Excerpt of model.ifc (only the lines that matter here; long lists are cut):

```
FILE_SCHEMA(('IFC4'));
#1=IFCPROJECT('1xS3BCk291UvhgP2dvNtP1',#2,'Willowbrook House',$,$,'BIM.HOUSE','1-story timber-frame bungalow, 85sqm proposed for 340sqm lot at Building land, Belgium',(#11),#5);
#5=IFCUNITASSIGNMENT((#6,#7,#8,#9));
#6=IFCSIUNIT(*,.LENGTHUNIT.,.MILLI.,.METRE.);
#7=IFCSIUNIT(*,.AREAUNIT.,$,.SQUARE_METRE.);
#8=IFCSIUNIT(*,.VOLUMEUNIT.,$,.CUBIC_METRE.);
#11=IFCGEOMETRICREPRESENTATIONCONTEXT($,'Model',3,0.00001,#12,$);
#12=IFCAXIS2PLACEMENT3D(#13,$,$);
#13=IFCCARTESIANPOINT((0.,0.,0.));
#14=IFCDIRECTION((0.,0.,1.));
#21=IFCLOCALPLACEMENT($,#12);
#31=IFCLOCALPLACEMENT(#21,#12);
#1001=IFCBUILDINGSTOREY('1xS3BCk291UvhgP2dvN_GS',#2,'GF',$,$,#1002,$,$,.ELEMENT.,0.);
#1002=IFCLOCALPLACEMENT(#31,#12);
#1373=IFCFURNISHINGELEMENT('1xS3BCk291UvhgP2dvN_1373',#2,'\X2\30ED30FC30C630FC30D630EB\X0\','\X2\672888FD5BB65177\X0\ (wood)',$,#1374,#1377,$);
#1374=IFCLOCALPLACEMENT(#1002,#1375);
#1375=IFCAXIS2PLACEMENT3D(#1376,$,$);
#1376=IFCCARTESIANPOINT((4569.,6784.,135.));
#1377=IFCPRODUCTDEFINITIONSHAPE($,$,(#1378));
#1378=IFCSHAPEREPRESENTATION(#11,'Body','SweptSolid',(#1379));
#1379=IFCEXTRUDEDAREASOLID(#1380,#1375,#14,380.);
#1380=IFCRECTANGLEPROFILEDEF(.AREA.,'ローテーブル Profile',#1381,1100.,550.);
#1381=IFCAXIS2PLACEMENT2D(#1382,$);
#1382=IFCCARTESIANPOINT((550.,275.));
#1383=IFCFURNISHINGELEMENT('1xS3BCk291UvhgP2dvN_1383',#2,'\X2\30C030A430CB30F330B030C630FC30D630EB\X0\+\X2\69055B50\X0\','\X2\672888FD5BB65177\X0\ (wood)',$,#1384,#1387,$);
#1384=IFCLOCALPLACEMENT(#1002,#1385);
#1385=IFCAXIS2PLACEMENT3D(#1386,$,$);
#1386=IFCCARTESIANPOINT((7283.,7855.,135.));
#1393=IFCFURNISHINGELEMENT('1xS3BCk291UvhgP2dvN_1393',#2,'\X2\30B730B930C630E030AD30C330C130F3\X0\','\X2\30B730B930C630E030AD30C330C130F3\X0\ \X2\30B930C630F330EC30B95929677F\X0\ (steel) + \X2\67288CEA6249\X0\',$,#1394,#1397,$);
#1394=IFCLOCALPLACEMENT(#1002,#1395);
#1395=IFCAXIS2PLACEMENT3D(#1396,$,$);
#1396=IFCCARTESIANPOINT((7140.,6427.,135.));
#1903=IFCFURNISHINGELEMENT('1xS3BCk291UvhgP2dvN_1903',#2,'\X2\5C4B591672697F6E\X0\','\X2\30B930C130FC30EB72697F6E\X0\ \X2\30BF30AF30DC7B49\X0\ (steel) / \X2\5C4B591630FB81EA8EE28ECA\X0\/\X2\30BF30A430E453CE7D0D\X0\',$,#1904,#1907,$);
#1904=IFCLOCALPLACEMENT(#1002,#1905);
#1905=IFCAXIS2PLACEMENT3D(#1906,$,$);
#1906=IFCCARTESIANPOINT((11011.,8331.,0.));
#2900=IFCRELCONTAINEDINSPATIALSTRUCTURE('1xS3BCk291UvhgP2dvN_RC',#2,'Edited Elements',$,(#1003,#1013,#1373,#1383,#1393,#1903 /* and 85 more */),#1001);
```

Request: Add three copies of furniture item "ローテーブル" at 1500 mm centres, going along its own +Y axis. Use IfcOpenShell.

```python
import ifcopenshell
import ifcopenshell.api.geometry
import ifcopenshell.api.root
import ifcopenshell.util.element
import ifcopenshell.util.placement

model = ifcopenshell.open("model.ifc")


def reuse_history(source, copy):
    """copy_class also copies each property set's owner history, people and application; keep the originals."""
    for rel in copy.IsDefinedBy:
        if rel.is_a("IfcRelDefinesByProperties") and (history := rel.RelatingPropertyDefinition.OwnerHistory):
            rel.RelatingPropertyDefinition.OwnerHistory = source.OwnerHistory
            ifcopenshell.util.element.remove_deep2(model, history)


source = model.by_guid("1xS3BCk291UvhgP2dvN_1373")
base = ifcopenshell.util.placement.get_local_placement(source.ObjectPlacement)
step = base[:3, 1] * 1500.0

for i in range(1, 4):
    copy = ifcopenshell.api.root.copy_class(model, product=source)
    copy.Representation = ifcopenshell.util.element.copy_deep(
        model, source.Representation, exclude=["IfcGeometricRepresentationContext", "IfcRepresentationMap"]
    )
    reuse_history(source, copy)
    matrix = base.copy()
    matrix[:3, 3] += i * step
    print("added at", matrix[:3, 3].round(3) + 0.0)
    ifcopenshell.api.geometry.edit_object_placement(model, product=copy, matrix=matrix, is_si=False)

model.write("model_edited.ifc")
```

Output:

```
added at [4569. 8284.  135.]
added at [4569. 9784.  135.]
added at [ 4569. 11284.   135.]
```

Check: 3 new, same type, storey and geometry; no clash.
